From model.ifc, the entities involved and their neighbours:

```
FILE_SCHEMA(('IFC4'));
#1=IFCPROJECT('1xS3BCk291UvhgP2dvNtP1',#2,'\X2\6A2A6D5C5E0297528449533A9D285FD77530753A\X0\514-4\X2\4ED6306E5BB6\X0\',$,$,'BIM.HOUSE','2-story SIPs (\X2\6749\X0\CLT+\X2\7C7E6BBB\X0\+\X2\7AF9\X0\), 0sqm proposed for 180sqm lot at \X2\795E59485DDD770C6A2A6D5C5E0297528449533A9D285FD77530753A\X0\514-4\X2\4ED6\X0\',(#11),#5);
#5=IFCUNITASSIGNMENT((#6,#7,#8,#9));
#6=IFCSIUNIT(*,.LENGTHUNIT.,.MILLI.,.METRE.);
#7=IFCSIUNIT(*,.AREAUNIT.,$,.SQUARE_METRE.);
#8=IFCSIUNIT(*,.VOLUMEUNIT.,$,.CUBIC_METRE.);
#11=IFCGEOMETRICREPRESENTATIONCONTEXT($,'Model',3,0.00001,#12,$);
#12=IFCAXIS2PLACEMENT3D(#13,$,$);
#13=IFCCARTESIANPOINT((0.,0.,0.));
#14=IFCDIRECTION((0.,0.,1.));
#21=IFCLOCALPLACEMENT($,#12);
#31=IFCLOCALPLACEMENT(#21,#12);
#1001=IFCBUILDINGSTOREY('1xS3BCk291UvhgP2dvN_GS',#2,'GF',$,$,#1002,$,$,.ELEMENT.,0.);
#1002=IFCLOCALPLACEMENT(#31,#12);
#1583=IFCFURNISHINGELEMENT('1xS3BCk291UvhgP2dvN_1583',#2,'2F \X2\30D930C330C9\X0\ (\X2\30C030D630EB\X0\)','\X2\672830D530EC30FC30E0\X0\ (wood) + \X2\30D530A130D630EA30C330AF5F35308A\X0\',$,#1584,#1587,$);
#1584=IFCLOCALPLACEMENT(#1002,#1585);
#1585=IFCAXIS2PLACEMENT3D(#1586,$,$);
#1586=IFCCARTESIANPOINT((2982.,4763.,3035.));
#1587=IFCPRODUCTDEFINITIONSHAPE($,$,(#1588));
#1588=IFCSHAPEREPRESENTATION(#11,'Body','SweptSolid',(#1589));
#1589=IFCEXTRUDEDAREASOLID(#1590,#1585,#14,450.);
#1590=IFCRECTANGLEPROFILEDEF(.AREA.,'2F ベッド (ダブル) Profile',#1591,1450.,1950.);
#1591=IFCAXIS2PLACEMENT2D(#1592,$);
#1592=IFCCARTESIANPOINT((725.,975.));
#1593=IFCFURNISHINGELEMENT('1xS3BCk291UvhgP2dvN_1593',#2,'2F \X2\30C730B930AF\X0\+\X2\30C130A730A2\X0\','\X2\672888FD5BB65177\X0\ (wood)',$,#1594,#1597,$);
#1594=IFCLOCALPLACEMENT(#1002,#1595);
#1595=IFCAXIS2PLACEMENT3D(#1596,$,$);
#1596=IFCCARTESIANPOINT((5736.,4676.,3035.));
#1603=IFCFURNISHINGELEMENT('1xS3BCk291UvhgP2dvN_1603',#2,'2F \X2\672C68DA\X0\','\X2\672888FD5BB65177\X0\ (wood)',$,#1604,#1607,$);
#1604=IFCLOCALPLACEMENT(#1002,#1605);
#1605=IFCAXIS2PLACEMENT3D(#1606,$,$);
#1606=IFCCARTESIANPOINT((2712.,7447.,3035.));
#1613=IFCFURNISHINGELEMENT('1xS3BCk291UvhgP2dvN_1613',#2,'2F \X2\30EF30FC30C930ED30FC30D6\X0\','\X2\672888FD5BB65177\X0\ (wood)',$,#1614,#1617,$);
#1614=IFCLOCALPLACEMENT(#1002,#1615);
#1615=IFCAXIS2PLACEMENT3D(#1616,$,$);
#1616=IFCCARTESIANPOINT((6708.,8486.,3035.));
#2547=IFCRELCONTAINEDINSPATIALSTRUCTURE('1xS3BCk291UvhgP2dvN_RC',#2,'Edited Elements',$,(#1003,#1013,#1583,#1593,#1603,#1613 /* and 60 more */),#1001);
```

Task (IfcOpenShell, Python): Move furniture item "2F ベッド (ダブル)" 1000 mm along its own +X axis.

```python
import ifcopenshell
import ifcopenshell.api.geometry
import ifcopenshell.util.placement
import ifcopenshell.util.unit

model = ifcopenshell.open("model.ifc")
unit_scale = ifcopenshell.util.unit.calculate_unit_scale(model)

item = model.by_id(1583)
matrix = ifcopenshell.util.placement.get_local_placement(item.ObjectPlacement)
matrix[:3, 3] += matrix[:3, 0] * 1 / unit_scale
ifcopenshell.api.geometry.edit_object_placement(model, product=item, matrix=matrix, is_si=False)

print(ifcopenshell.util.placement.get_local_placement(item.ObjectPlacement).round(3) + 0.0)

model.write("model-out.ifc")
```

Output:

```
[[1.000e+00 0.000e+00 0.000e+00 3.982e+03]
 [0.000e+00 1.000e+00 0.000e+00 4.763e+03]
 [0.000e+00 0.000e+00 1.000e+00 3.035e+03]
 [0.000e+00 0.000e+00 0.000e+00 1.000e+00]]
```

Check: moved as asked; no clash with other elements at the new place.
